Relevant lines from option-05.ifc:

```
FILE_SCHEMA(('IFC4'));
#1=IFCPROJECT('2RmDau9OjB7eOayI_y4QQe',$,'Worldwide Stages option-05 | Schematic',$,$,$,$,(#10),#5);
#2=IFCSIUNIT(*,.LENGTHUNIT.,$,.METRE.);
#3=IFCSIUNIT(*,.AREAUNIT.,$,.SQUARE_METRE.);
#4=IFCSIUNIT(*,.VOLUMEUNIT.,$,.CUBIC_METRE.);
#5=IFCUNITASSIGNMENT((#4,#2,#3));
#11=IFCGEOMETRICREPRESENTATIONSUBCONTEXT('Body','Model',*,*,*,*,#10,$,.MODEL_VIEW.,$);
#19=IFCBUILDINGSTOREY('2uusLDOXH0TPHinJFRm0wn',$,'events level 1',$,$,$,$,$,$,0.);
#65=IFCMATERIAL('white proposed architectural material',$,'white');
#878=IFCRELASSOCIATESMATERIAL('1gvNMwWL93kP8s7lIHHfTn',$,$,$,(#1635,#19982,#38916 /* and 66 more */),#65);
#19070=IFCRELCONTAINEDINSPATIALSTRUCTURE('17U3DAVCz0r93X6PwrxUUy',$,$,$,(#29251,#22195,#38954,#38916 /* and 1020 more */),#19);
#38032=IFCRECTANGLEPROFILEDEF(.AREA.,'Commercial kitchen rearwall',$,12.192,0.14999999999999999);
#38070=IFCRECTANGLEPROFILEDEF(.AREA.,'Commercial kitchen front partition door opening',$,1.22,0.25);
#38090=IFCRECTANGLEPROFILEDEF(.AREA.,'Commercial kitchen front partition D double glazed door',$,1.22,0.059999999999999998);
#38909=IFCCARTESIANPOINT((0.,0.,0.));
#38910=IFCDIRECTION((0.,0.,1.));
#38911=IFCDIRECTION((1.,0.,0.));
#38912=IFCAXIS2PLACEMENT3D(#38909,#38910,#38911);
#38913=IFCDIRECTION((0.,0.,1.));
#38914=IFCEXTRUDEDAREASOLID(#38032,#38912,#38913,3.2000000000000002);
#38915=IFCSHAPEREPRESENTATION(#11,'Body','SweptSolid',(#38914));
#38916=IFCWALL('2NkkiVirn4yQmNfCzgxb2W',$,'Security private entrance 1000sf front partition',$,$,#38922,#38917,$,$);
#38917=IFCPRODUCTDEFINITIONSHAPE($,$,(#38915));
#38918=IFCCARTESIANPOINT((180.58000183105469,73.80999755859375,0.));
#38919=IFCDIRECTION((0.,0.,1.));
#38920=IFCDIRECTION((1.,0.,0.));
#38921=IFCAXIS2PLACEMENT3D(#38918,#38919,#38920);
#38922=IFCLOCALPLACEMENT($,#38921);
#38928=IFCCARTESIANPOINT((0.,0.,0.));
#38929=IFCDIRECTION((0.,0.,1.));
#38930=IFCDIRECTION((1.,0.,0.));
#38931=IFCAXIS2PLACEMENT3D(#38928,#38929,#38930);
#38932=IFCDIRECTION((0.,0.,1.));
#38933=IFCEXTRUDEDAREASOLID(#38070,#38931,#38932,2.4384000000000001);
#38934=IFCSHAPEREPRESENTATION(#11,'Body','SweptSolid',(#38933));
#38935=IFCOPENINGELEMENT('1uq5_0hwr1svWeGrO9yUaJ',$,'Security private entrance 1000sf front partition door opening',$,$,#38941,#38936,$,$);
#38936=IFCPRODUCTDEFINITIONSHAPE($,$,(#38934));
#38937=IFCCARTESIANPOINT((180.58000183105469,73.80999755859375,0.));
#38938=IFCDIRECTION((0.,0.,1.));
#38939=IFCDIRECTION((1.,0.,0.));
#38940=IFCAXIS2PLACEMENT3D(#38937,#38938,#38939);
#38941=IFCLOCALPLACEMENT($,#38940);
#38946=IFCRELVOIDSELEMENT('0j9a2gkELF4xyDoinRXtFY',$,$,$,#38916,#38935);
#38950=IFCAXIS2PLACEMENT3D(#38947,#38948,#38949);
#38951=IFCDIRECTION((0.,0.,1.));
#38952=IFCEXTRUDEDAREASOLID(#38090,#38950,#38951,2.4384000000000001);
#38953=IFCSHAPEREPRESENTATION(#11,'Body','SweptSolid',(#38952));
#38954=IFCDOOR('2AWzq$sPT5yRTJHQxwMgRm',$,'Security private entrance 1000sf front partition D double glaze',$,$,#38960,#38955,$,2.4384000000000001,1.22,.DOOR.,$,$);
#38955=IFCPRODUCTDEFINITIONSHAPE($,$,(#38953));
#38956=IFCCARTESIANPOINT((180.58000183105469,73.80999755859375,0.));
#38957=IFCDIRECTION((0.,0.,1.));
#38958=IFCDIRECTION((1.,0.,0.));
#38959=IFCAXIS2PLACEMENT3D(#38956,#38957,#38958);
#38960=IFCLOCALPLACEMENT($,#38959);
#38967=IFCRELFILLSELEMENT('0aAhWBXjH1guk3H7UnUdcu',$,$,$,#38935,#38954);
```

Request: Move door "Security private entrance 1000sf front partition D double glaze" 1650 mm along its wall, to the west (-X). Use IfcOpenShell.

```python
import ifcopenshell
import ifcopenshell.api.geometry
import ifcopenshell.util.placement
import ifcopenshell.util.unit

model = ifcopenshell.open("option-05.ifc")
unit_scale = ifcopenshell.util.unit.calculate_unit_scale(model)

door = model.by_guid("2AWzq$sPT5yRTJHQxwMgRm")
opening = door.FillsVoids[0].RelatingOpeningElement
wall = opening.VoidsElements[0].RelatingBuildingElement

wall_matrix = ifcopenshell.util.placement.get_local_placement(wall.ObjectPlacement)
shift = wall_matrix[:3, 0] * -1.65 / unit_scale
before = ifcopenshell.util.placement.get_local_placement(door.ObjectPlacement)[:3, 3].copy()

# The door is not placed relative to its opening, so move both.
for product in (opening, door):
    matrix = ifcopenshell.util.placement.get_local_placement(product.ObjectPlacement)
    matrix[:3, 3] += shift
    ifcopenshell.api.geometry.edit_object_placement(model, product=product, matrix=matrix, is_si=False)

after = ifcopenshell.util.placement.get_local_placement(door.ObjectPlacement)[:3, 3]
print("door moved by", (after - before).round(3) + 0.0)

model.write("option-05_updated.ifc")
```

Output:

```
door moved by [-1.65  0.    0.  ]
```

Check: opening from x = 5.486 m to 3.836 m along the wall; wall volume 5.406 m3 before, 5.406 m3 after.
